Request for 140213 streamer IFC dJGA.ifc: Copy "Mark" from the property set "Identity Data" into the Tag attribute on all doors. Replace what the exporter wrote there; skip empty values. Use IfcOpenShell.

First a look at what the model holds.

```python
import ifcopenshell
import ifcopenshell.util.element

model = ifcopenshell.open("140213 streamer IFC dJGA.ifc")
print(model.schema)
doors = model.by_type("IfcDoor")
print(len(doors), "doors")
for e in doors[:8]:
    source = ifcopenshell.util.element.get_pset(e, "Identity Data", "Mark")
    target = e.Tag
    print(e.id(), repr(source), repr(target), sep=" | ")
```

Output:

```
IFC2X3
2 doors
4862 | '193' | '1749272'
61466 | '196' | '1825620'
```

```python
import ifcopenshell
import ifcopenshell.util.element

model = ifcopenshell.open("140213 streamer IFC dJGA.ifc")

count = 0
for e in model.by_type("IfcDoor"):
    value = ifcopenshell.util.element.get_pset(e, "Identity Data", "Mark")
    current = e.Tag
    if not value or not value.strip() or current == value:
        continue
    e.Tag = value
    count += 1

print(count, "doors updated")

model.write("140213 streamer IFC dJGA_v2.ifc")
```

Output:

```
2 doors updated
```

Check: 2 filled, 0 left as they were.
